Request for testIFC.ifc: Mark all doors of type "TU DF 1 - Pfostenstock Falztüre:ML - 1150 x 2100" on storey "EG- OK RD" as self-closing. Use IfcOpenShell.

First a look at what the model holds.

```python
import ifcopenshell
import ifcopenshell.util.element

model = ifcopenshell.open("testIFC.ifc")
print(model.schema)
storey = next(s for s in model.by_type("IfcBuildingStorey") if s.Name == "EG- OK RD")
doors = [e for e in ifcopenshell.util.element.get_decomposition(storey) if e.is_a("IfcDoor")]
seen = {}
for e in doors:
    element_type = ifcopenshell.util.element.get_type(e)
    key = (element_type.Name if element_type != e and element_type else None, ifcopenshell.util.element.get_pset(e, "Pset_DoorCommon", "SelfClosing"))
    seen[key] = seen.get(key, 0) + 1
for (name, value), count in sorted(seen.items(), key=str):
    print(count, "x", name, "|", value)
```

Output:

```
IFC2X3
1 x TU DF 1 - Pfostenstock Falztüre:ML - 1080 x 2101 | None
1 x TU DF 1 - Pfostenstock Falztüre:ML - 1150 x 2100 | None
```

```python
import ifcopenshell
import ifcopenshell.api.pset
import ifcopenshell.util.element

model = ifcopenshell.open("testIFC.ifc")

storey = next(s for s in model.by_type("IfcBuildingStorey") if s.Name == "EG- OK RD")
doors = [e for e in ifcopenshell.util.element.get_decomposition(storey) if e.is_a("IfcDoor")]

count = 0
for e in doors:
    element_type = ifcopenshell.util.element.get_type(e)
    if element_type in (None, e) or element_type.Name != "TU DF 1 - Pfostenstock Falztüre:ML - 1150 x 2100":
        continue
    # add_pset returns the element's existing set when there is one.
    pset = ifcopenshell.api.pset.add_pset(model, product=e, name="Pset_DoorCommon")
    ifcopenshell.api.pset.edit_pset(model, pset=pset, properties={"SelfClosing": True})
    count += 1

print(count, "doors updated")

model.write("testIFC_updated.ifc")
```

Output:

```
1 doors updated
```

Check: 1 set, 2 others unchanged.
